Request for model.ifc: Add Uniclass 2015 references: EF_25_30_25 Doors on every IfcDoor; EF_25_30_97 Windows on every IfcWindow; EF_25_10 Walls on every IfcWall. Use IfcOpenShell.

First a look at what the model holds.

```python
import ifcopenshell

model = ifcopenshell.open("model.ifc")
print(model.schema)
print("classifications:", [c.Name for c in model.by_type("IfcClassification")])
for ifc_class in ("IfcDoor", "IfcRoof", "IfcStair", "IfcWall", "IfcWindow"):
    print(ifc_class, len(model.by_type(ifc_class)))
```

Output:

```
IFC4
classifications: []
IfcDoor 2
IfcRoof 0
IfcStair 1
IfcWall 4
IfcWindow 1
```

```python
import ifcopenshell
import ifcopenshell.api.classification

model = ifcopenshell.open("model.ifc")

system = ifcopenshell.api.classification.add_classification(model, classification="Uniclass 2015")

codes = {
    "IfcDoor": ("EF_25_30_25", "Doors"),
    "IfcWindow": ("EF_25_30_97", "Windows"),
    "IfcWall": ("EF_25_10", "Walls"),
}
for ifc_class, (code, name) in codes.items():
    products = model.by_type(ifc_class)
    ifcopenshell.api.classification.add_reference(
        model, products=products, classification=system, identification=code, name=name
    )
    print(code, len(products))

model.write("model_rev.ifc")
```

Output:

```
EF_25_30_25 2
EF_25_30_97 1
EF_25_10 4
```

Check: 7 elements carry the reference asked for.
